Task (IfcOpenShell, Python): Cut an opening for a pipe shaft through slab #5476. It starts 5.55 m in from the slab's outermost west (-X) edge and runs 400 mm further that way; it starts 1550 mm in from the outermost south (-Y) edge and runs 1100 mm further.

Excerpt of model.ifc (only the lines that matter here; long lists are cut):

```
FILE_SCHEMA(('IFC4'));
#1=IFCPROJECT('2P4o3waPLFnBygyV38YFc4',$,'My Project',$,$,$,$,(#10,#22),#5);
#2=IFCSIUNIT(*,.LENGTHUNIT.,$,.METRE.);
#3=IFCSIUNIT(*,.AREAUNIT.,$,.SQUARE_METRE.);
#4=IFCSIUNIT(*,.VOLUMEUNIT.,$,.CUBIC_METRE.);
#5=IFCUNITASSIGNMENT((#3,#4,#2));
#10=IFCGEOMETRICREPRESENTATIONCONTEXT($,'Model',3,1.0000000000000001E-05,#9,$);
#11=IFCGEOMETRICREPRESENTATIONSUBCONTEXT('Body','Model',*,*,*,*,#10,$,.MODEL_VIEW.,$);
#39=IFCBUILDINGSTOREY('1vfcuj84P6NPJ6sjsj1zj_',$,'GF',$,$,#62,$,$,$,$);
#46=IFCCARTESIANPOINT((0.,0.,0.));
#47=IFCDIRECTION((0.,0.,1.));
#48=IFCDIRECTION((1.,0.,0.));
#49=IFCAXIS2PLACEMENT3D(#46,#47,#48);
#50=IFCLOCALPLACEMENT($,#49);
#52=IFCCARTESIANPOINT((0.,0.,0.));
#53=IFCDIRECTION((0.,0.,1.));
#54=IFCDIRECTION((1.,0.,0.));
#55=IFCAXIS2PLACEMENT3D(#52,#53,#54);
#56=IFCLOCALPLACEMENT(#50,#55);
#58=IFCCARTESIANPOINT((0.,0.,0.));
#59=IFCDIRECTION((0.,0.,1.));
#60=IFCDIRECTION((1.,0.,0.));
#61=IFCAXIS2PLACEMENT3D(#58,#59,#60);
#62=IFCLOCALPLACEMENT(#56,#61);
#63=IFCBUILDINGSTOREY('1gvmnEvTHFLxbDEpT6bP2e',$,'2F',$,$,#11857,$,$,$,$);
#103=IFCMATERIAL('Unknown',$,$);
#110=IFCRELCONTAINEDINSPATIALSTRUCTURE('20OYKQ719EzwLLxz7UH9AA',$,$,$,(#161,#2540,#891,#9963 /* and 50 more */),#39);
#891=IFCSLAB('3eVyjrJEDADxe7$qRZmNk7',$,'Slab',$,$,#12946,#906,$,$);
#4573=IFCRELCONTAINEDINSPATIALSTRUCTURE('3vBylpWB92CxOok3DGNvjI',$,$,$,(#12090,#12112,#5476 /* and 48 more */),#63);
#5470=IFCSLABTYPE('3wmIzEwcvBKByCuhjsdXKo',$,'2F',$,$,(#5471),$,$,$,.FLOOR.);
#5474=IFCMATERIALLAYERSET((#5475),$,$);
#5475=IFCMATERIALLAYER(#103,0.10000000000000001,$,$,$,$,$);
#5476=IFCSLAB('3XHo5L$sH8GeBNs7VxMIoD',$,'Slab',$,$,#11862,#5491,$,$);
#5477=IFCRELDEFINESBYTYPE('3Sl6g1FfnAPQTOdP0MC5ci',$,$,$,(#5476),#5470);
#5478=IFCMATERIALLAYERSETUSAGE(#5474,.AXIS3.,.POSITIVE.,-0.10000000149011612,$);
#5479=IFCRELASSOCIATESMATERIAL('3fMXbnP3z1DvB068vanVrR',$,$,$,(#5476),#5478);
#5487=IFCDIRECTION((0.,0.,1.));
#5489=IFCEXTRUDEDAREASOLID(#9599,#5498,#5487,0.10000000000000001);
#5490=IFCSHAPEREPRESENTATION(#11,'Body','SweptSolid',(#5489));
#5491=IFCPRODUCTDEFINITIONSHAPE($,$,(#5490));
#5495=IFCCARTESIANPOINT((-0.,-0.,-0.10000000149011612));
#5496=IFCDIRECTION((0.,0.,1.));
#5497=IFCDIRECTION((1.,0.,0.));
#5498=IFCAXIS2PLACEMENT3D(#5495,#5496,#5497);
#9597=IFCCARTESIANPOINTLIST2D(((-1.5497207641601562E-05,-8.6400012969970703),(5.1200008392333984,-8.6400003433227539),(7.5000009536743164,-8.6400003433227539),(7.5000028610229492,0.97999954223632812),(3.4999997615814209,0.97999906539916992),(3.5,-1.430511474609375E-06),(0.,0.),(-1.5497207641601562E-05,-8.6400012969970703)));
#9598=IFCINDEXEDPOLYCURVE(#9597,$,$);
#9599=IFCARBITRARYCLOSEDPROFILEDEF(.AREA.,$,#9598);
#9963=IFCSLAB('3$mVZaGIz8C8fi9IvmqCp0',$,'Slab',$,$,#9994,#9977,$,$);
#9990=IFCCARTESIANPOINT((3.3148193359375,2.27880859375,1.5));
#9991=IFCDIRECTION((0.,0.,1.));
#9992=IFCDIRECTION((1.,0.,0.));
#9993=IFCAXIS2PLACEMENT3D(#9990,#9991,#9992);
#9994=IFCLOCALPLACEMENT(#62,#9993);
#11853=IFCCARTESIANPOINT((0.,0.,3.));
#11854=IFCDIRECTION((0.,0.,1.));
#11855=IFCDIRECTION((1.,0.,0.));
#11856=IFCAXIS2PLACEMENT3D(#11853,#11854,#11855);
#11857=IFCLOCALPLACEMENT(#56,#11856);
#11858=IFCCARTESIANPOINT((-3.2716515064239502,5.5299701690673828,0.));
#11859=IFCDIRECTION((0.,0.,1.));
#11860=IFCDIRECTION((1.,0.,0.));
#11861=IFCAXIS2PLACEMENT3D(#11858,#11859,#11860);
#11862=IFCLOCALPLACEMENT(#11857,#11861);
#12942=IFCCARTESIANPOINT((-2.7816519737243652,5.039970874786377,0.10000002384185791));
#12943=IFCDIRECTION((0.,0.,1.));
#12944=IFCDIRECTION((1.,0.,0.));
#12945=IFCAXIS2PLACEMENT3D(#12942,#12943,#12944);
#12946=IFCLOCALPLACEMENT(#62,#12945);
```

```python
import numpy as np
import ifcopenshell
import ifcopenshell.api.feature
import ifcopenshell.api.geometry
import ifcopenshell.api.root
import ifcopenshell.geom
import ifcopenshell.util.placement
import ifcopenshell.util.representation
import ifcopenshell.util.shape
import ifcopenshell.util.unit

model = ifcopenshell.open("model.ifc")
unit_scale = ifcopenshell.util.unit.calculate_unit_scale(model)
settings = ifcopenshell.geom.settings()


def volume(element):
    """Net volume in cubic metres, openings subtracted."""
    shape = ifcopenshell.geom.create_shape(settings, element)
    return ifcopenshell.util.shape.get_volume(shape.geometry)


slab = model.by_id(5476)
before = volume(slab)

# Extent in the slab's own axes, in metres. The edges named are its -X and -Y sides.
slab_shape = ifcopenshell.geom.create_shape(settings, slab)
vertices = ifcopenshell.util.shape.get_vertices(slab_shape.geometry)
x_min, y_min, bottom = vertices.min(axis=0)
top = vertices[:, 2].max()

opening = ifcopenshell.api.root.create_entity(model, ifc_class="IfcOpeningElement", name="Pipe shaft opening", predefined_type="OPENING")
context = ifcopenshell.util.representation.get_context(model, "Model", "Body", "MODEL_VIEW")
width, depth = 0.4, 1.1
outline = [(0.0, 0.0), (width, 0.0), (width, depth), (0.0, depth), (0.0, 0.0)]
# Overshoot both faces by 50 mm so the cut is clean.
shape = ifcopenshell.api.geometry.add_slab_representation(
    model, context=context, depth=top - bottom + 0.1, polyline=outline
)
ifcopenshell.api.geometry.assign_representation(model, product=opening, representation=shape)

matrix = ifcopenshell.util.placement.get_local_placement(slab.ObjectPlacement)
matrix[:, 3] = matrix @ np.append(np.array([x_min + 5.55, y_min + 1.55, bottom - 0.05]) / unit_scale, 1.0)
ifcopenshell.api.geometry.edit_object_placement(model, product=opening, matrix=matrix, is_si=False)
ifcopenshell.api.feature.add_feature(model, feature=opening, element=slab)

after = volume(slab)

print(f"slab volume {before:.3f} -> {after:.3f} m3")

model.write("model-out.ifc")
```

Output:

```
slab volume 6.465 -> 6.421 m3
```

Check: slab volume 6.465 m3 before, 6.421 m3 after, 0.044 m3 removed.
